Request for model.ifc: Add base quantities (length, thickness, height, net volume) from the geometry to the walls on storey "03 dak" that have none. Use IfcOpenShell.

First a look at what the model holds.

```python
import ifcopenshell
import ifcopenshell.util.element
import ifcopenshell.util.unit

model = ifcopenshell.open("model.ifc")
print(model.schema)
for unit_type in ("LENGTHUNIT", "AREAUNIT", "VOLUMEUNIT"):
    print(unit_type, ifcopenshell.util.unit.calculate_unit_scale(model, unit_type))
storey = next(s for s in model.by_type("IfcBuildingStorey") if s.Name == "03 dak")
walls = [e for e in ifcopenshell.util.element.get_decomposition(storey) if e.is_a("IfcWall")]
for e in sorted(walls, key=lambda e: e.id()):
    print(e.id(), e.is_a(), e.Name, list(ifcopenshell.util.element.get_psets(e, qtos_only=True)), sep=" | ")
```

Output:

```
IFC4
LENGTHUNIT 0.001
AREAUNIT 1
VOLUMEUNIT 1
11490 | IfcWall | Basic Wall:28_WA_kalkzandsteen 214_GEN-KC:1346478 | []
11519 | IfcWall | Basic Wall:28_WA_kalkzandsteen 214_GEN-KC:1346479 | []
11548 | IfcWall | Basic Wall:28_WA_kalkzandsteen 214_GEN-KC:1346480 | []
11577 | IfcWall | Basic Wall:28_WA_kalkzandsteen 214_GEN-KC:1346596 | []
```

```python
import ifcopenshell
import ifcopenshell.api.pset
import ifcopenshell.geom
import ifcopenshell.util.element
import ifcopenshell.util.shape
import ifcopenshell.util.unit

model = ifcopenshell.open("model.ifc")
unit_scale = ifcopenshell.util.unit.calculate_unit_scale(model)
volume_scale = ifcopenshell.util.unit.calculate_unit_scale(model, "VOLUMEUNIT")
settings = ifcopenshell.geom.settings()

storey = next(s for s in model.by_type("IfcBuildingStorey") if s.Name == "03 dak")
walls = [e for e in ifcopenshell.util.element.get_decomposition(storey) if e.is_a("IfcWall")]

for e in sorted(walls, key=lambda e: e.id()):
    if ifcopenshell.util.element.get_psets(e, qtos_only=True, should_inherit=False):
        continue
    # Geometry comes back in metres, in the element's own axes.
    shape = ifcopenshell.geom.create_shape(settings, e)
    values = {
        "Length": ifcopenshell.util.shape.get_x(shape.geometry) / unit_scale,
        "Width": ifcopenshell.util.shape.get_y(shape.geometry) / unit_scale,
        "Height": ifcopenshell.util.shape.get_z(shape.geometry) / unit_scale,
        "NetVolume": ifcopenshell.util.shape.get_volume(shape.geometry) / volume_scale,
    }
    qto = ifcopenshell.api.pset.add_qto(model, product=e, name="Qto_WallBaseQuantities")
    ifcopenshell.api.pset.edit_qto(model, qto=qto, properties=values)
    print(e.id(), {k: round(v, 3) for k, v in values.items()})

model.write("model_updated.ifc")
```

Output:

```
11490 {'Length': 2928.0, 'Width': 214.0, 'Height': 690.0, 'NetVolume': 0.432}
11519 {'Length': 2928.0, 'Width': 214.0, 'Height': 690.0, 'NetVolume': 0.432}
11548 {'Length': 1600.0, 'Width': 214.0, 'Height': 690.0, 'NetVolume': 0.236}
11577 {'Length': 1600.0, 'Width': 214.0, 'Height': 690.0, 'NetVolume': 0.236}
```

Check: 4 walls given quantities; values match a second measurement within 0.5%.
